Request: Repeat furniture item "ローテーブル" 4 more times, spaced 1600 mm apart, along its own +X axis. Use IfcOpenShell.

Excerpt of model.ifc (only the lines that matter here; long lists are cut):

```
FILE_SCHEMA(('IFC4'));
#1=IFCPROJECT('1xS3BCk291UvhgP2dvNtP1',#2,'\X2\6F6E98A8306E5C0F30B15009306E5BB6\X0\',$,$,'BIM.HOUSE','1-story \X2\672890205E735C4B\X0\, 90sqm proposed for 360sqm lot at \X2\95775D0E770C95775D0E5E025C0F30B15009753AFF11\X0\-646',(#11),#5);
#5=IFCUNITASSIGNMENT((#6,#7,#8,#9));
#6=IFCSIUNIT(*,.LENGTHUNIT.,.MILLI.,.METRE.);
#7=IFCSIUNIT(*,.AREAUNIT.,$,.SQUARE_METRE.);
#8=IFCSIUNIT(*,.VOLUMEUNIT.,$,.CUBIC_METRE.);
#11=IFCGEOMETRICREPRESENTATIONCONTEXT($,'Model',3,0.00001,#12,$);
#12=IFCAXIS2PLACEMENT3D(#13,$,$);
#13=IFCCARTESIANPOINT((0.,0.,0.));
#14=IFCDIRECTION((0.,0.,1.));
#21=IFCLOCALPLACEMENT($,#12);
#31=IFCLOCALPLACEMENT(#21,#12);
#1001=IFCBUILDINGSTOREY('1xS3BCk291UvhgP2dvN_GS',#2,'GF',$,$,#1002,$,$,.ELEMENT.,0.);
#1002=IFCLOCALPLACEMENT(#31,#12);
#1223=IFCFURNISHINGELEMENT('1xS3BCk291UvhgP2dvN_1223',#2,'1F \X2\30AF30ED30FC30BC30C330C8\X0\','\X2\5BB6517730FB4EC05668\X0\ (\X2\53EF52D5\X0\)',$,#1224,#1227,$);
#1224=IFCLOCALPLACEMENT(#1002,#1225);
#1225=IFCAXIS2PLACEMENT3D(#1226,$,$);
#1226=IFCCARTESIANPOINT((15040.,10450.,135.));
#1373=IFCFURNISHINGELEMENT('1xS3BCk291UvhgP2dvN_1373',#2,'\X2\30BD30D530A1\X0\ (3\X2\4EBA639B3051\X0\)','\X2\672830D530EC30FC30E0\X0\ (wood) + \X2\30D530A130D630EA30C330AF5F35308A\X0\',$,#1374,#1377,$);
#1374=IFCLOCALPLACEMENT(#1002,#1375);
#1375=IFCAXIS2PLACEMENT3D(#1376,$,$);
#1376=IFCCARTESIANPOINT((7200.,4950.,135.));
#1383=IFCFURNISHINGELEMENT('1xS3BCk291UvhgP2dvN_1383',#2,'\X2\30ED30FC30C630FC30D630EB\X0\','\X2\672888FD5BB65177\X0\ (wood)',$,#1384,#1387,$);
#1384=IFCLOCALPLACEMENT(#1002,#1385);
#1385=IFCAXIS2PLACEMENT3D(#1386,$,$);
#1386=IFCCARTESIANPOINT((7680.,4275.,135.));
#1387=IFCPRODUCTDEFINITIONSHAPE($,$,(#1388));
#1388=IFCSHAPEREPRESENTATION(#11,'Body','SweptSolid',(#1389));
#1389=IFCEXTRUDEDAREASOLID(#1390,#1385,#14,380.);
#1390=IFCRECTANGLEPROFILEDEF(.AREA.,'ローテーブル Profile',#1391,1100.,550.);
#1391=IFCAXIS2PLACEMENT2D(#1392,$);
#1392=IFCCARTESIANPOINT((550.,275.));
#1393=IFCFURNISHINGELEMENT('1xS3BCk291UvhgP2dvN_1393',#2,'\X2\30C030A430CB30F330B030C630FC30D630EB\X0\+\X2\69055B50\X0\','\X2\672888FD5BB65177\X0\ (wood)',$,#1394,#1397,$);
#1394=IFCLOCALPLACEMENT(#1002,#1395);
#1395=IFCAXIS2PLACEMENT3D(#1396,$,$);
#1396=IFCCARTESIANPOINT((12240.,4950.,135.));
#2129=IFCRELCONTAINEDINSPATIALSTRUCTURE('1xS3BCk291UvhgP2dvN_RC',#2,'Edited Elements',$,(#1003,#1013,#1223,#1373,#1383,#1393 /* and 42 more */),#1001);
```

```python
import ifcopenshell
import ifcopenshell.api.geometry
import ifcopenshell.api.root
import ifcopenshell.util.element
import ifcopenshell.util.placement
import ifcopenshell.util.unit

model = ifcopenshell.open("model.ifc")
unit_scale = ifcopenshell.util.unit.calculate_unit_scale(model)


def reuse_history(source, copy):
    """copy_class also copies each property set's owner history, people and application; keep the originals."""
    for rel in copy.IsDefinedBy:
        if rel.is_a("IfcRelDefinesByProperties") and (history := rel.RelatingPropertyDefinition.OwnerHistory):
            rel.RelatingPropertyDefinition.OwnerHistory = source.OwnerHistory
            ifcopenshell.util.element.remove_deep2(model, history)


source = model.by_guid("1xS3BCk291UvhgP2dvN_1383")
base = ifcopenshell.util.placement.get_local_placement(source.ObjectPlacement)
step = base[:3, 0] * 1.6 / unit_scale

for i in range(1, 5):
    copy = ifcopenshell.api.root.copy_class(model, product=source)
    copy.Representation = ifcopenshell.util.element.copy_deep(
        model, source.Representation, exclude=["IfcGeometricRepresentationContext", "IfcRepresentationMap"]
    )
    reuse_history(source, copy)
    matrix = base.copy()
    matrix[:3, 3] += i * step
    print("added at", matrix[:3, 3].round(3) + 0.0)
    ifcopenshell.api.geometry.edit_object_placement(model, product=copy, matrix=matrix, is_si=False)

model.write("model_updated.ifc")
```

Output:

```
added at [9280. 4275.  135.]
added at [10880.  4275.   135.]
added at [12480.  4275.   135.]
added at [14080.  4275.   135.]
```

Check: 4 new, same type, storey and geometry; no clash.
